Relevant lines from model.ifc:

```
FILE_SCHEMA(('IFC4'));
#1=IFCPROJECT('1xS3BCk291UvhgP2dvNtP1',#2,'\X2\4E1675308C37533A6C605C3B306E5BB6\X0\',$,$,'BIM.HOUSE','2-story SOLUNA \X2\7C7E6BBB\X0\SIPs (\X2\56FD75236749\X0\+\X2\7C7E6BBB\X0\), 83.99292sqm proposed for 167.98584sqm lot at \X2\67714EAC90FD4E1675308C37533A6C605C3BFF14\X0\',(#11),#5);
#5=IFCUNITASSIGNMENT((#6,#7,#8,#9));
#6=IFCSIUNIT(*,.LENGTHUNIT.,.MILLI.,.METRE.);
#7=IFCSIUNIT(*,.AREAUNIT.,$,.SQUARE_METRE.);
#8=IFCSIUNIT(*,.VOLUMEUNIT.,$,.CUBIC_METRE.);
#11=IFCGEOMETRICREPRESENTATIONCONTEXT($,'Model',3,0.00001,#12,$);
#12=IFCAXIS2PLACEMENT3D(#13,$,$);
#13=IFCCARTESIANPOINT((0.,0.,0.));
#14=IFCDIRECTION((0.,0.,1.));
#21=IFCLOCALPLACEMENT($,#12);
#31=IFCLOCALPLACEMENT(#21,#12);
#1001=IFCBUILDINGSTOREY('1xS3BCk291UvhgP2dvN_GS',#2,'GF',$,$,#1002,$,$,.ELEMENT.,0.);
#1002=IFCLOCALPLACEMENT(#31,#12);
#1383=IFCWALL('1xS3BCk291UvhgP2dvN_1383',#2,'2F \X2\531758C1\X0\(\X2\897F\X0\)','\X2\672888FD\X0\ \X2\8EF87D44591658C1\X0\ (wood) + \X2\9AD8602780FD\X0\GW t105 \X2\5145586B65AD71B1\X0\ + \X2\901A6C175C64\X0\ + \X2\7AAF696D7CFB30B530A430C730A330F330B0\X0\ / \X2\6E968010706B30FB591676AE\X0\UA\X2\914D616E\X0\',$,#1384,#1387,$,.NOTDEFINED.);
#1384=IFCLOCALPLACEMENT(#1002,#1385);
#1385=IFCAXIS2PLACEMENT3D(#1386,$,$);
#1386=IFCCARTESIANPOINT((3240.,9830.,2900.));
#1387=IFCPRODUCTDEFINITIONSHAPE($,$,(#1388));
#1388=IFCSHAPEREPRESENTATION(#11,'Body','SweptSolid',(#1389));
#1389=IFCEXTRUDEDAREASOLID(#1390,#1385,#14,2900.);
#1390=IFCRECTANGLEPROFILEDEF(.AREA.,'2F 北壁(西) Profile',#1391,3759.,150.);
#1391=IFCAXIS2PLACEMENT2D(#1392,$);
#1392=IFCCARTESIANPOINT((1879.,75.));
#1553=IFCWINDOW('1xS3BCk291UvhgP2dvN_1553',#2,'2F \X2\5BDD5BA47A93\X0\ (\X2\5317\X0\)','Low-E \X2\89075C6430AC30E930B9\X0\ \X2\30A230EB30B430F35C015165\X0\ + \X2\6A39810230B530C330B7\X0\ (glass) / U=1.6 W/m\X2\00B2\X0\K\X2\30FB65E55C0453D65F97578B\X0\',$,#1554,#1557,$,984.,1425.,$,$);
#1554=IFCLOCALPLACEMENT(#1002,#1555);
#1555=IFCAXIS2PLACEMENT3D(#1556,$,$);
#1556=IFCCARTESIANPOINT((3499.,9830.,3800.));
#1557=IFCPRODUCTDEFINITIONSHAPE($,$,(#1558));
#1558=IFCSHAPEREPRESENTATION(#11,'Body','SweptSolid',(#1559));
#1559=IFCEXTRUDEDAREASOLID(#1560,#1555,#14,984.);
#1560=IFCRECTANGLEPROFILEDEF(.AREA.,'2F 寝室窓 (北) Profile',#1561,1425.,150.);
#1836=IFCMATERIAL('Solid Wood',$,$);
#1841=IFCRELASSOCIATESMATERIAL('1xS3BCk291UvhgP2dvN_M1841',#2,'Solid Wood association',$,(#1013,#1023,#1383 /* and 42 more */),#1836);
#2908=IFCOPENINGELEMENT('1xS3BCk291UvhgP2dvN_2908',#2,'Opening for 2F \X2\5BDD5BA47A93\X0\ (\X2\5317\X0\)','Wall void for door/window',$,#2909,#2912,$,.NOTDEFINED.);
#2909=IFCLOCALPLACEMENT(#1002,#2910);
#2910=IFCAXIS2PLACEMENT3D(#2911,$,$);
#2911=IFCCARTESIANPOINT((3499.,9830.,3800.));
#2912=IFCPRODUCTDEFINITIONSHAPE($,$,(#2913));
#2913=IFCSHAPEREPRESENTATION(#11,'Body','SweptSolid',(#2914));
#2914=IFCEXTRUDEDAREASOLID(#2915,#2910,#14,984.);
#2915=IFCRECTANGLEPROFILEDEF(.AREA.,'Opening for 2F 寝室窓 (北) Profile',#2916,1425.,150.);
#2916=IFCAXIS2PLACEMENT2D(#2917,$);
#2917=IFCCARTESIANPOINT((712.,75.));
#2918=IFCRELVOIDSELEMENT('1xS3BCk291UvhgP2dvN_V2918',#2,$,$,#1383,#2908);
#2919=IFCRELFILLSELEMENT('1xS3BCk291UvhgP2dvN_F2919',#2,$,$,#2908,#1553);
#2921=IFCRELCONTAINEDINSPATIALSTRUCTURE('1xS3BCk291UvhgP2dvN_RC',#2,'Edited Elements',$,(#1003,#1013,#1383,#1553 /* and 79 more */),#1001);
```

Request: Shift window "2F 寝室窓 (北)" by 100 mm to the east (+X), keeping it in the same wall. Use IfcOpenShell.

```python
import ifcopenshell
import ifcopenshell.api.geometry
import ifcopenshell.util.placement

model = ifcopenshell.open("model.ifc")

window = model.by_guid("1xS3BCk291UvhgP2dvN_1553")
opening = window.FillsVoids[0].RelatingOpeningElement
wall = opening.VoidsElements[0].RelatingBuildingElement

wall_matrix = ifcopenshell.util.placement.get_local_placement(wall.ObjectPlacement)
shift = wall_matrix[:3, 0] * 100.0
before = ifcopenshell.util.placement.get_local_placement(window.ObjectPlacement)[:3, 3].copy()

# The window is not placed relative to its opening, so move both.
for product in (opening, window):
    matrix = ifcopenshell.util.placement.get_local_placement(product.ObjectPlacement)
    matrix[:3, 3] += shift
    ifcopenshell.api.geometry.edit_object_placement(model, product=product, matrix=matrix, is_si=False)

after = ifcopenshell.util.placement.get_local_placement(window.ObjectPlacement)[:3, 3]
print("window moved by", (after - before).round(3) + 0.0)

model.write("model-out.ifc")
```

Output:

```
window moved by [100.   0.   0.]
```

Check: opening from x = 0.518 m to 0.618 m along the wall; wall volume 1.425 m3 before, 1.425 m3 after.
